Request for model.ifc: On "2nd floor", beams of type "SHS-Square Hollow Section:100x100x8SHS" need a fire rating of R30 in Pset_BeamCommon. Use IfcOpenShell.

First a look at what the model holds.

```python
import ifcopenshell
import ifcopenshell.util.element

model = ifcopenshell.open("model.ifc")
print(model.schema)
storey = next(s for s in model.by_type("IfcBuildingStorey") if s.Name == "2nd floor")
beams = [e for e in ifcopenshell.util.element.get_decomposition(storey) if e.is_a("IfcBeam")]
seen = {}
for e in beams:
    element_type = ifcopenshell.util.element.get_type(e)
    key = (element_type.Name if element_type != e and element_type else None, ifcopenshell.util.element.get_pset(e, "Pset_BeamCommon", "FireRating"))
    seen[key] = seen.get(key, 0) + 1
for (name, value), count in sorted(seen.items(), key=str):
    print(count, "x", name, "|", value)
```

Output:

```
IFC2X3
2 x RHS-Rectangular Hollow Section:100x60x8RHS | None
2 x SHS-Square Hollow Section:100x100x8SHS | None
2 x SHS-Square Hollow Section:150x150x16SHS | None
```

```python
import ifcopenshell
import ifcopenshell.api.pset
import ifcopenshell.util.element

model = ifcopenshell.open("model.ifc")

storey = next(s for s in model.by_type("IfcBuildingStorey") if s.Name == "2nd floor")
beams = [e for e in ifcopenshell.util.element.get_decomposition(storey) if e.is_a("IfcBeam")]

count = 0
for e in beams:
    element_type = ifcopenshell.util.element.get_type(e)
    if element_type in (None, e) or element_type.Name != "SHS-Square Hollow Section:100x100x8SHS":
        continue
    # add_pset returns the element's existing set when there is one.
    pset = ifcopenshell.api.pset.add_pset(model, product=e, name="Pset_BeamCommon")
    ifcopenshell.api.pset.edit_pset(model, pset=pset, properties={"FireRating": "R30"})
    count += 1

print(count, "beams updated")

model.write("model_updated.ifc")
```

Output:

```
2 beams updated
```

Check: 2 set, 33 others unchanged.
